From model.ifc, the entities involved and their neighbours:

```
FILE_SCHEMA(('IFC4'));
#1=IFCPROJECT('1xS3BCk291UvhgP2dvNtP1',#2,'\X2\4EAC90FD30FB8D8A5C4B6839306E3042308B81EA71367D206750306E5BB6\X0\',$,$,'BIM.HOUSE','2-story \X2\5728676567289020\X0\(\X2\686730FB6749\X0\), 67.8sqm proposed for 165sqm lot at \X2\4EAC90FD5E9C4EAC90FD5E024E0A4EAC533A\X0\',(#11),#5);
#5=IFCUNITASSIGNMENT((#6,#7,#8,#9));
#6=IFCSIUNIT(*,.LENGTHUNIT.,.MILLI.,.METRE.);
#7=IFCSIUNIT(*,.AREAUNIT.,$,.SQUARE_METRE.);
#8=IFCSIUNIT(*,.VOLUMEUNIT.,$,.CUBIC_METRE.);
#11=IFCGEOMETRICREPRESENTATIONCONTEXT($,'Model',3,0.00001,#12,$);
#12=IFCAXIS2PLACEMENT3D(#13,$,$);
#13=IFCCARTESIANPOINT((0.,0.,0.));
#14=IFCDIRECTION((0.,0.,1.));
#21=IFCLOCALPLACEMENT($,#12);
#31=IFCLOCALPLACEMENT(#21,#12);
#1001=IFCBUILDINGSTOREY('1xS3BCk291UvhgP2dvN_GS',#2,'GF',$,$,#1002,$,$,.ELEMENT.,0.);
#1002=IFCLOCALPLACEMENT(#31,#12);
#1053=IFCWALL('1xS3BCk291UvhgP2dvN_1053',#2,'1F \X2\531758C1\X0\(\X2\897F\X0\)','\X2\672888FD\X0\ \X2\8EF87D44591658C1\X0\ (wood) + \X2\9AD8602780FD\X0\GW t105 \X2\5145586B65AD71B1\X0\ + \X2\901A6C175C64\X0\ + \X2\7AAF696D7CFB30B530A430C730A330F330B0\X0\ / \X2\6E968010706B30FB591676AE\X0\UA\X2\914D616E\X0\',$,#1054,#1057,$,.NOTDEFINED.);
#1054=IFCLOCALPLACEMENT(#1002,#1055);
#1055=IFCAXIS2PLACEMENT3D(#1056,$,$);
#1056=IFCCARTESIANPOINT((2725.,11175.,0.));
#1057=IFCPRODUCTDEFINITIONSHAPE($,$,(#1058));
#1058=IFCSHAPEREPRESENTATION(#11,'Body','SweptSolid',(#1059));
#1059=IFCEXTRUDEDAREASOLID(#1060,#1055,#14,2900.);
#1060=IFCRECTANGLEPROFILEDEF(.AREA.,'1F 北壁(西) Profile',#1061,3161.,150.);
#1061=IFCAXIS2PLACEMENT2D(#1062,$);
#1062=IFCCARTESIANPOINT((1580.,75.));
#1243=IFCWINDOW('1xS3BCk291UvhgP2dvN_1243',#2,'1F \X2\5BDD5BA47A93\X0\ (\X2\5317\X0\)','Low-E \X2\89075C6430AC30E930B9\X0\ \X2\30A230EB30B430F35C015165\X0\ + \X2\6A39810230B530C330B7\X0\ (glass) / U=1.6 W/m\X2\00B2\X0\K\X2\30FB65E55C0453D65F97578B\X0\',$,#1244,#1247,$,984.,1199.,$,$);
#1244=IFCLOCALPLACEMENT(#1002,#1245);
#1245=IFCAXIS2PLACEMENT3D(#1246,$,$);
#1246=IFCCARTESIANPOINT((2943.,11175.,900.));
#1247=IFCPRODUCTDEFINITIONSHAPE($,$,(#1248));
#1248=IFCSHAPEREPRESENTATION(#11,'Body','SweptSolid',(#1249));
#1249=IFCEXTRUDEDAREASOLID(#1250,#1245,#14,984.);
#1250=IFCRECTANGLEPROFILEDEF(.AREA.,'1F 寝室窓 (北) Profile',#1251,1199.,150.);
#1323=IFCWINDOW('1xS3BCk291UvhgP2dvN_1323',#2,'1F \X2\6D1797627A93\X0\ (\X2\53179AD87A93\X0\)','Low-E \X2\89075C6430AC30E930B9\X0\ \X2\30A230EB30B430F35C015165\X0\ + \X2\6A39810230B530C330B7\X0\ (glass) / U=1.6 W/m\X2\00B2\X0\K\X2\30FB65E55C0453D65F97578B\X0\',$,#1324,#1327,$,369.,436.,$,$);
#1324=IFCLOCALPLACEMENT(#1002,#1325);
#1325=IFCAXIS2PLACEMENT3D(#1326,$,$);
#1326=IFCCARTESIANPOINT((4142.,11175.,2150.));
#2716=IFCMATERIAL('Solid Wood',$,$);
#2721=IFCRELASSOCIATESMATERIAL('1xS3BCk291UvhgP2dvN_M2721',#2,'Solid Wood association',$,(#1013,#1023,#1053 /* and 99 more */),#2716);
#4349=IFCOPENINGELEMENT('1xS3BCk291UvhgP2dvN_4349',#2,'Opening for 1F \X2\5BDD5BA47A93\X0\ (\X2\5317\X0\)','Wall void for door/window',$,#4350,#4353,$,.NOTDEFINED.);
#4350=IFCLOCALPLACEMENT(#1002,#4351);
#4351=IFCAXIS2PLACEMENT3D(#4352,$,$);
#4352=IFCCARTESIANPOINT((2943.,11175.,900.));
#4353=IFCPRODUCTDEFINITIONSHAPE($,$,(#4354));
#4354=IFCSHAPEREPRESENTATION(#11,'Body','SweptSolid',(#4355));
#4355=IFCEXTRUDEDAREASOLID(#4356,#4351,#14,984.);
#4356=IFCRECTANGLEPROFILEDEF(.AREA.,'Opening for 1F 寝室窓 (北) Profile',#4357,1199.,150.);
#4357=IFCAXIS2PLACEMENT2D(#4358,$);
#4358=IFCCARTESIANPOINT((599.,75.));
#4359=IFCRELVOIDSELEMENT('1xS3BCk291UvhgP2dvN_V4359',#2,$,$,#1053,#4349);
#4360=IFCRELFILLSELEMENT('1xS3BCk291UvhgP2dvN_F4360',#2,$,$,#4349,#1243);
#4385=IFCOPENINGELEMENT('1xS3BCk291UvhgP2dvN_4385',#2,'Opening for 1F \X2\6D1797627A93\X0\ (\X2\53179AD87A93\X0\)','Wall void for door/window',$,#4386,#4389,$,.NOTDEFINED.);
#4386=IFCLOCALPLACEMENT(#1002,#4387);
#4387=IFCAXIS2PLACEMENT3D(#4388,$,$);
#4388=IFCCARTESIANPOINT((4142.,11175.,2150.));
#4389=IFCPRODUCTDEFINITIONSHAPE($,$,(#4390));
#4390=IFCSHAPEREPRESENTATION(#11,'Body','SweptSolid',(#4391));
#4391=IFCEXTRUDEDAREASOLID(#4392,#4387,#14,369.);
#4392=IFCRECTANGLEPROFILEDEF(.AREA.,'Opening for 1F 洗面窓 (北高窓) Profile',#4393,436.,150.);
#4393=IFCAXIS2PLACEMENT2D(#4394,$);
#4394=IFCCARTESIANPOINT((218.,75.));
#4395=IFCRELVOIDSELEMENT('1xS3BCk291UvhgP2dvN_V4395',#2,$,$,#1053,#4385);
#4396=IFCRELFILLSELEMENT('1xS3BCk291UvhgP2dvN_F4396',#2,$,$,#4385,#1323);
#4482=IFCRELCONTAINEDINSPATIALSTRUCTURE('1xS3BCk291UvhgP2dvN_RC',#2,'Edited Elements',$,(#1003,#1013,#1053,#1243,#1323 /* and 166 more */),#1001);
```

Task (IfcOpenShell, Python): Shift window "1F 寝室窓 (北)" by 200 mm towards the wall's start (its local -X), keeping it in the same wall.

```python
import ifcopenshell
import ifcopenshell.api.geometry
import ifcopenshell.util.placement
import ifcopenshell.util.unit

model = ifcopenshell.open("model.ifc")
unit_scale = ifcopenshell.util.unit.calculate_unit_scale(model)

window = model.by_guid("1xS3BCk291UvhgP2dvN_1243")
opening = window.FillsVoids[0].RelatingOpeningElement
wall = opening.VoidsElements[0].RelatingBuildingElement

wall_matrix = ifcopenshell.util.placement.get_local_placement(wall.ObjectPlacement)
shift = wall_matrix[:3, 0] * -0.2 / unit_scale
before = ifcopenshell.util.placement.get_local_placement(window.ObjectPlacement)[:3, 3].copy()

# The window is not placed relative to its opening, so move both.
for product in (opening, window):
    matrix = ifcopenshell.util.placement.get_local_placement(product.ObjectPlacement)
    matrix[:3, 3] += shift
    ifcopenshell.api.geometry.edit_object_placement(model, product=product, matrix=matrix, is_si=False)

after = ifcopenshell.util.placement.get_local_placement(window.ObjectPlacement)[:3, 3]
print("window moved by", (after - before).round(3) + 0.0)

model.write("model_updated.ifc")
```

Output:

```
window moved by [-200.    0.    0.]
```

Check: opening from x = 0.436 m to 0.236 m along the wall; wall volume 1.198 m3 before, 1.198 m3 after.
